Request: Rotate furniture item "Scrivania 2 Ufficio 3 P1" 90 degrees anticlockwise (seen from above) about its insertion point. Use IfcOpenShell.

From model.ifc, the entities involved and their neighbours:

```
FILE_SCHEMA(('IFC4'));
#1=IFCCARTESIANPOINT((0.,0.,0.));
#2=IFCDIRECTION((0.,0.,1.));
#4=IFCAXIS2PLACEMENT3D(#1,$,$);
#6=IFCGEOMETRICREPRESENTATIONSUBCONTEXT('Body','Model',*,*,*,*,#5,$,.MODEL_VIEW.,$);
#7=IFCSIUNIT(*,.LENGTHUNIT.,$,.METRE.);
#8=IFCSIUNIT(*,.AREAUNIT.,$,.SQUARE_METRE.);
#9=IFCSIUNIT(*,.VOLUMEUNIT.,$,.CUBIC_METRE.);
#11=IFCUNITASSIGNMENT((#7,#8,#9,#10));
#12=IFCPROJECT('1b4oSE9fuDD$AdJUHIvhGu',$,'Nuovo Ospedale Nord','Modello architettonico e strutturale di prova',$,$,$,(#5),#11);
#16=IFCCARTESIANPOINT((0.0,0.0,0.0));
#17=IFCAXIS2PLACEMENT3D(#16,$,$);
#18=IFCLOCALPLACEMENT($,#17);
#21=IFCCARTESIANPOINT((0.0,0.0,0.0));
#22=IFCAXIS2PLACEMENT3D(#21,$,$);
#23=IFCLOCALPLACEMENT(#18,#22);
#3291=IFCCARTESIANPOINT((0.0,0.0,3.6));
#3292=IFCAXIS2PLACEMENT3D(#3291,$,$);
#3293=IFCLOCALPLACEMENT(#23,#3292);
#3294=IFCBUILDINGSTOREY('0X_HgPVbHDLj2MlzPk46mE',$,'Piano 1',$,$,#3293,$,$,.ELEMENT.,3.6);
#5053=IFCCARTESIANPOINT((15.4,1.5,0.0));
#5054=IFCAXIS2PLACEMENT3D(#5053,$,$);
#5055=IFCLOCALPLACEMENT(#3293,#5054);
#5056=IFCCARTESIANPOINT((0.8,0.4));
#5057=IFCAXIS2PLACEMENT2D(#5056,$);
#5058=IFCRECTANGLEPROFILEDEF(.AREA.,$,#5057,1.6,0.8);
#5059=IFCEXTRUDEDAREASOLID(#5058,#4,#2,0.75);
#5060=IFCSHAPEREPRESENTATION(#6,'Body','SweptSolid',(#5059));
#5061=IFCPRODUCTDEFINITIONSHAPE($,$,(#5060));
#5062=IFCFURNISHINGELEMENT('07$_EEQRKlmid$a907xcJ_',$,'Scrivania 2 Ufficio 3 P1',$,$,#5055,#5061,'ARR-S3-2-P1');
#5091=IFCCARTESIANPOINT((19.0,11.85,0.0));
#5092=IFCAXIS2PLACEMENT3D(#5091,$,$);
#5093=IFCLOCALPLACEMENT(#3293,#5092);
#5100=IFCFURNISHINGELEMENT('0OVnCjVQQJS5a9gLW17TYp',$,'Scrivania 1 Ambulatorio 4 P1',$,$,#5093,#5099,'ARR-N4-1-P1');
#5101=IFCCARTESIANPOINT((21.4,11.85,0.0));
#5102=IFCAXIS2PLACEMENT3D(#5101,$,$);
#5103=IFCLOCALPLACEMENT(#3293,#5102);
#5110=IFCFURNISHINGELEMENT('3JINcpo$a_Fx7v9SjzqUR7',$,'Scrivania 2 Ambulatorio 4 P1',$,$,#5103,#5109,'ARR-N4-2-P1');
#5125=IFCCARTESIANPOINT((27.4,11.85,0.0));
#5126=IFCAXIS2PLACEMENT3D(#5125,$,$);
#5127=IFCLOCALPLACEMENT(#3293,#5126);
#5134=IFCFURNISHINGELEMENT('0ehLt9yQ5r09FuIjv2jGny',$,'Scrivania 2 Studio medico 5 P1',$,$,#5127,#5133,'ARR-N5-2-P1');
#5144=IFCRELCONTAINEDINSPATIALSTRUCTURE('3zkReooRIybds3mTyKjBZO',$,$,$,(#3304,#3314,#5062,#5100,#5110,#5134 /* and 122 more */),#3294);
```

```python
import ifcopenshell
import ifcopenshell.api.geometry
import ifcopenshell.util.placement

model = ifcopenshell.open("model.ifc")

item = model.by_guid("07$_EEQRKlmid$a907xcJ_")
matrix = ifcopenshell.util.placement.get_local_placement(item.ObjectPlacement)
matrix = matrix @ ifcopenshell.util.placement.rotation(90, "Z")
ifcopenshell.api.geometry.edit_object_placement(model, product=item, matrix=matrix, is_si=False)

print(ifcopenshell.util.placement.get_local_placement(item.ObjectPlacement).round(3) + 0.0)

model.write("model_rev.ifc")
```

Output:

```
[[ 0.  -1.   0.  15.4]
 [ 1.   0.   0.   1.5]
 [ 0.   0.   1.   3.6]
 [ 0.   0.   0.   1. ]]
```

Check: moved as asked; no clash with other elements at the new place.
